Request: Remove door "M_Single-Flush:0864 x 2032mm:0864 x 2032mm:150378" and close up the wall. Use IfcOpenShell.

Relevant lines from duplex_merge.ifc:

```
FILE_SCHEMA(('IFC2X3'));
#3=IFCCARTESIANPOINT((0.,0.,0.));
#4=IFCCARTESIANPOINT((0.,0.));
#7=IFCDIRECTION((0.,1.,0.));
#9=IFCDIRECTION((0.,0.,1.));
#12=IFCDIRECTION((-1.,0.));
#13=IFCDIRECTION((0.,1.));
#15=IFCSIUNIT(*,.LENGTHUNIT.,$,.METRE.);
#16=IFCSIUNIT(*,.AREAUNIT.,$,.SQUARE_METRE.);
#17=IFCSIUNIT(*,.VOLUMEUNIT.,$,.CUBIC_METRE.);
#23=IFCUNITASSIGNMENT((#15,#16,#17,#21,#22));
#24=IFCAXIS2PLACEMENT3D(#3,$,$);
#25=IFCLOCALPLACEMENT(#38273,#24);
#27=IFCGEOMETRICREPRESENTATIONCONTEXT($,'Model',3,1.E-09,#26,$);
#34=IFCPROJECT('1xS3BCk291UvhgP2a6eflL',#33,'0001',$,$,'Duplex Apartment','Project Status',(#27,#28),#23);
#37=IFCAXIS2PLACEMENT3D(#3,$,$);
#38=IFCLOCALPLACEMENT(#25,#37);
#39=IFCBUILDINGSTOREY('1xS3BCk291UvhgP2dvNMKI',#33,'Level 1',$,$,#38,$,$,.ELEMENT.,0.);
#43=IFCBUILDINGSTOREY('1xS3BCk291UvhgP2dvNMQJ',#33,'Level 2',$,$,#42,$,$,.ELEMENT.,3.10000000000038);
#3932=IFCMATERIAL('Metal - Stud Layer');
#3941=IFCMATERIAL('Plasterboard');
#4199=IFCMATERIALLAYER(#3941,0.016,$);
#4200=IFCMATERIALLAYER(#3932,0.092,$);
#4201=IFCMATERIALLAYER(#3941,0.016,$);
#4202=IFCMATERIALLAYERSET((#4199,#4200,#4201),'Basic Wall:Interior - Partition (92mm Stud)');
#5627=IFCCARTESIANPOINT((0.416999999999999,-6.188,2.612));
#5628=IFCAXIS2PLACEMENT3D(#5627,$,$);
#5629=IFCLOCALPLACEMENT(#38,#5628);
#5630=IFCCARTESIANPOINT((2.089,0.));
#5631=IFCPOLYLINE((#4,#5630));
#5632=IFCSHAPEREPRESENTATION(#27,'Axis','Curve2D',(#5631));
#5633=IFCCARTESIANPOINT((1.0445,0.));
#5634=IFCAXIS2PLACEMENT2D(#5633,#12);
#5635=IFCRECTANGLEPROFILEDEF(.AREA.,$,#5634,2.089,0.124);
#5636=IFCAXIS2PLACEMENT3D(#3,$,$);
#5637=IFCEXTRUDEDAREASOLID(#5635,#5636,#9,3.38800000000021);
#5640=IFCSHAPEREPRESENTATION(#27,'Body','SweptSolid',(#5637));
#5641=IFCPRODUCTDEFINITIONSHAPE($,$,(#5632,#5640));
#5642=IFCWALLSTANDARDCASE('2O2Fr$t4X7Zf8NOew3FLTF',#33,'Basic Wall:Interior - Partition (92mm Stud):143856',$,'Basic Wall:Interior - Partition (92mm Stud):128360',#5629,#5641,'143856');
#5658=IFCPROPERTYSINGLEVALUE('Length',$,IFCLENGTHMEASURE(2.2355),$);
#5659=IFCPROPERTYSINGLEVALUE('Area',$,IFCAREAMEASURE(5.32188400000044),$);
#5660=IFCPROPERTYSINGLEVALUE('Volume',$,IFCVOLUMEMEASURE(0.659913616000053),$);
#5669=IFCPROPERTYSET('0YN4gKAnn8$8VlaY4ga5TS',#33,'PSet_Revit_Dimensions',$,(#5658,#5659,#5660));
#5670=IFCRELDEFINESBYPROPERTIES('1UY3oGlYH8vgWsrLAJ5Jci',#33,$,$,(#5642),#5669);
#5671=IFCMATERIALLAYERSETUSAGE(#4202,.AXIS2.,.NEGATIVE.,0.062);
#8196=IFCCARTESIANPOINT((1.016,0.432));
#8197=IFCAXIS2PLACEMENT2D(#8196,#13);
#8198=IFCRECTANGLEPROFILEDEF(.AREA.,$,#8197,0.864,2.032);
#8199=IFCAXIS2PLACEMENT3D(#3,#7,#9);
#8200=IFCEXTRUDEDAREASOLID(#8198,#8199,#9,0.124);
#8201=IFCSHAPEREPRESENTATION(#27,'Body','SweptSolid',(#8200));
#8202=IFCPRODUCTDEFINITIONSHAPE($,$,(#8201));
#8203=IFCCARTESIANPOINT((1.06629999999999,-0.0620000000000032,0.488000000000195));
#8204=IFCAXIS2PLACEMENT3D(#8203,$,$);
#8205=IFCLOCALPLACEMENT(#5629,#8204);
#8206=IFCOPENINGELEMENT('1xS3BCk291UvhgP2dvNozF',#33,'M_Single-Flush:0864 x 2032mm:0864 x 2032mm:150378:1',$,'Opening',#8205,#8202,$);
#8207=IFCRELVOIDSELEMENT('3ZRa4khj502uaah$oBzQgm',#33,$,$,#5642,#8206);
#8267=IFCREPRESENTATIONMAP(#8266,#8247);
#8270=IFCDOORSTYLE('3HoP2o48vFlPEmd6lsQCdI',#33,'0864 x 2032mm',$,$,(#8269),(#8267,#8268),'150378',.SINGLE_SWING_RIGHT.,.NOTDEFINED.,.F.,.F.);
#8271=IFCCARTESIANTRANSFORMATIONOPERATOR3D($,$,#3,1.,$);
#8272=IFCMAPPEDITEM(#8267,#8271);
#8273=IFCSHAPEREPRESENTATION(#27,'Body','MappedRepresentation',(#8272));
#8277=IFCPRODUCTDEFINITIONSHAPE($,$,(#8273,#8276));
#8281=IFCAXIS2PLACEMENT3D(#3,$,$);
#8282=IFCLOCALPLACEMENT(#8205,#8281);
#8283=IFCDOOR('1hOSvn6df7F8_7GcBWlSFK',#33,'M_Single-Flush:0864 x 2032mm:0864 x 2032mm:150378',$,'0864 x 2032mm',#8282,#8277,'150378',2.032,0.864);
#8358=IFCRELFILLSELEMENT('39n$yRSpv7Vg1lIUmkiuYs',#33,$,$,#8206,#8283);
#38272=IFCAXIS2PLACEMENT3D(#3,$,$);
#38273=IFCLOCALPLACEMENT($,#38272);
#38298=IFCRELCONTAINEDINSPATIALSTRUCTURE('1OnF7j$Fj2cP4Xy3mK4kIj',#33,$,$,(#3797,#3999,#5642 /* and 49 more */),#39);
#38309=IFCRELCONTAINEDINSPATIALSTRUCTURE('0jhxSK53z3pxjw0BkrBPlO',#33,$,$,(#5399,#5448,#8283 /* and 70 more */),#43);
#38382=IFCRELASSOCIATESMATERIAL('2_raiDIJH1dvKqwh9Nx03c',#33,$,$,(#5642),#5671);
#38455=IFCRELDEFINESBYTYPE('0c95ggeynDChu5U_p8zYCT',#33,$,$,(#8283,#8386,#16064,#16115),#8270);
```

```python
import ifcopenshell
import ifcopenshell.api.feature
import ifcopenshell.api.pset
import ifcopenshell.api.root
import ifcopenshell.geom
import ifcopenshell.util.element
import ifcopenshell.util.shape
import ifcopenshell.util.unit

model = ifcopenshell.open("duplex_merge.ifc")
area_scale = ifcopenshell.util.unit.calculate_unit_scale(model, "AREAUNIT")
volume_scale = ifcopenshell.util.unit.calculate_unit_scale(model, "VOLUMEUNIT")
settings = ifcopenshell.geom.settings()


def volume(element):
    """Net volume in cubic metres, openings subtracted."""
    shape = ifcopenshell.geom.create_shape(settings, element)
    return ifcopenshell.util.shape.get_volume(shape.geometry)


door = model.by_guid("1hOSvn6df7F8_7GcBWlSFK")
opening = door.FillsVoids[0].RelatingOpeningElement
wall = opening.VoidsElements[0].RelatingBuildingElement
before = volume(wall)

ifcopenshell.api.root.remove_product(model, product=door)
ifcopenshell.api.feature.remove_feature(model, feature=opening)

after = volume(wall)
thickness = 0.124  # wall thickness in metres

# Update the wall's stored quantities.
pset = model.by_id(ifcopenshell.util.element.get_pset(wall, "PSet_Revit_Dimensions", should_inherit=False)["id"])
ifcopenshell.api.pset.edit_pset(model, pset=pset, properties={
    "Area": model.create_entity("IfcAreaMeasure", after / thickness / area_scale),
    "Volume": model.create_entity("IfcVolumeMeasure", after / volume_scale),
})

print(f"wall volume {before:.3f} -> {after:.3f} m3")

model.write("duplex_merge_rev.ifc")
```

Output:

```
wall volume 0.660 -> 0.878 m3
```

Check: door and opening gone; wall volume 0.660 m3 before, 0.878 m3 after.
